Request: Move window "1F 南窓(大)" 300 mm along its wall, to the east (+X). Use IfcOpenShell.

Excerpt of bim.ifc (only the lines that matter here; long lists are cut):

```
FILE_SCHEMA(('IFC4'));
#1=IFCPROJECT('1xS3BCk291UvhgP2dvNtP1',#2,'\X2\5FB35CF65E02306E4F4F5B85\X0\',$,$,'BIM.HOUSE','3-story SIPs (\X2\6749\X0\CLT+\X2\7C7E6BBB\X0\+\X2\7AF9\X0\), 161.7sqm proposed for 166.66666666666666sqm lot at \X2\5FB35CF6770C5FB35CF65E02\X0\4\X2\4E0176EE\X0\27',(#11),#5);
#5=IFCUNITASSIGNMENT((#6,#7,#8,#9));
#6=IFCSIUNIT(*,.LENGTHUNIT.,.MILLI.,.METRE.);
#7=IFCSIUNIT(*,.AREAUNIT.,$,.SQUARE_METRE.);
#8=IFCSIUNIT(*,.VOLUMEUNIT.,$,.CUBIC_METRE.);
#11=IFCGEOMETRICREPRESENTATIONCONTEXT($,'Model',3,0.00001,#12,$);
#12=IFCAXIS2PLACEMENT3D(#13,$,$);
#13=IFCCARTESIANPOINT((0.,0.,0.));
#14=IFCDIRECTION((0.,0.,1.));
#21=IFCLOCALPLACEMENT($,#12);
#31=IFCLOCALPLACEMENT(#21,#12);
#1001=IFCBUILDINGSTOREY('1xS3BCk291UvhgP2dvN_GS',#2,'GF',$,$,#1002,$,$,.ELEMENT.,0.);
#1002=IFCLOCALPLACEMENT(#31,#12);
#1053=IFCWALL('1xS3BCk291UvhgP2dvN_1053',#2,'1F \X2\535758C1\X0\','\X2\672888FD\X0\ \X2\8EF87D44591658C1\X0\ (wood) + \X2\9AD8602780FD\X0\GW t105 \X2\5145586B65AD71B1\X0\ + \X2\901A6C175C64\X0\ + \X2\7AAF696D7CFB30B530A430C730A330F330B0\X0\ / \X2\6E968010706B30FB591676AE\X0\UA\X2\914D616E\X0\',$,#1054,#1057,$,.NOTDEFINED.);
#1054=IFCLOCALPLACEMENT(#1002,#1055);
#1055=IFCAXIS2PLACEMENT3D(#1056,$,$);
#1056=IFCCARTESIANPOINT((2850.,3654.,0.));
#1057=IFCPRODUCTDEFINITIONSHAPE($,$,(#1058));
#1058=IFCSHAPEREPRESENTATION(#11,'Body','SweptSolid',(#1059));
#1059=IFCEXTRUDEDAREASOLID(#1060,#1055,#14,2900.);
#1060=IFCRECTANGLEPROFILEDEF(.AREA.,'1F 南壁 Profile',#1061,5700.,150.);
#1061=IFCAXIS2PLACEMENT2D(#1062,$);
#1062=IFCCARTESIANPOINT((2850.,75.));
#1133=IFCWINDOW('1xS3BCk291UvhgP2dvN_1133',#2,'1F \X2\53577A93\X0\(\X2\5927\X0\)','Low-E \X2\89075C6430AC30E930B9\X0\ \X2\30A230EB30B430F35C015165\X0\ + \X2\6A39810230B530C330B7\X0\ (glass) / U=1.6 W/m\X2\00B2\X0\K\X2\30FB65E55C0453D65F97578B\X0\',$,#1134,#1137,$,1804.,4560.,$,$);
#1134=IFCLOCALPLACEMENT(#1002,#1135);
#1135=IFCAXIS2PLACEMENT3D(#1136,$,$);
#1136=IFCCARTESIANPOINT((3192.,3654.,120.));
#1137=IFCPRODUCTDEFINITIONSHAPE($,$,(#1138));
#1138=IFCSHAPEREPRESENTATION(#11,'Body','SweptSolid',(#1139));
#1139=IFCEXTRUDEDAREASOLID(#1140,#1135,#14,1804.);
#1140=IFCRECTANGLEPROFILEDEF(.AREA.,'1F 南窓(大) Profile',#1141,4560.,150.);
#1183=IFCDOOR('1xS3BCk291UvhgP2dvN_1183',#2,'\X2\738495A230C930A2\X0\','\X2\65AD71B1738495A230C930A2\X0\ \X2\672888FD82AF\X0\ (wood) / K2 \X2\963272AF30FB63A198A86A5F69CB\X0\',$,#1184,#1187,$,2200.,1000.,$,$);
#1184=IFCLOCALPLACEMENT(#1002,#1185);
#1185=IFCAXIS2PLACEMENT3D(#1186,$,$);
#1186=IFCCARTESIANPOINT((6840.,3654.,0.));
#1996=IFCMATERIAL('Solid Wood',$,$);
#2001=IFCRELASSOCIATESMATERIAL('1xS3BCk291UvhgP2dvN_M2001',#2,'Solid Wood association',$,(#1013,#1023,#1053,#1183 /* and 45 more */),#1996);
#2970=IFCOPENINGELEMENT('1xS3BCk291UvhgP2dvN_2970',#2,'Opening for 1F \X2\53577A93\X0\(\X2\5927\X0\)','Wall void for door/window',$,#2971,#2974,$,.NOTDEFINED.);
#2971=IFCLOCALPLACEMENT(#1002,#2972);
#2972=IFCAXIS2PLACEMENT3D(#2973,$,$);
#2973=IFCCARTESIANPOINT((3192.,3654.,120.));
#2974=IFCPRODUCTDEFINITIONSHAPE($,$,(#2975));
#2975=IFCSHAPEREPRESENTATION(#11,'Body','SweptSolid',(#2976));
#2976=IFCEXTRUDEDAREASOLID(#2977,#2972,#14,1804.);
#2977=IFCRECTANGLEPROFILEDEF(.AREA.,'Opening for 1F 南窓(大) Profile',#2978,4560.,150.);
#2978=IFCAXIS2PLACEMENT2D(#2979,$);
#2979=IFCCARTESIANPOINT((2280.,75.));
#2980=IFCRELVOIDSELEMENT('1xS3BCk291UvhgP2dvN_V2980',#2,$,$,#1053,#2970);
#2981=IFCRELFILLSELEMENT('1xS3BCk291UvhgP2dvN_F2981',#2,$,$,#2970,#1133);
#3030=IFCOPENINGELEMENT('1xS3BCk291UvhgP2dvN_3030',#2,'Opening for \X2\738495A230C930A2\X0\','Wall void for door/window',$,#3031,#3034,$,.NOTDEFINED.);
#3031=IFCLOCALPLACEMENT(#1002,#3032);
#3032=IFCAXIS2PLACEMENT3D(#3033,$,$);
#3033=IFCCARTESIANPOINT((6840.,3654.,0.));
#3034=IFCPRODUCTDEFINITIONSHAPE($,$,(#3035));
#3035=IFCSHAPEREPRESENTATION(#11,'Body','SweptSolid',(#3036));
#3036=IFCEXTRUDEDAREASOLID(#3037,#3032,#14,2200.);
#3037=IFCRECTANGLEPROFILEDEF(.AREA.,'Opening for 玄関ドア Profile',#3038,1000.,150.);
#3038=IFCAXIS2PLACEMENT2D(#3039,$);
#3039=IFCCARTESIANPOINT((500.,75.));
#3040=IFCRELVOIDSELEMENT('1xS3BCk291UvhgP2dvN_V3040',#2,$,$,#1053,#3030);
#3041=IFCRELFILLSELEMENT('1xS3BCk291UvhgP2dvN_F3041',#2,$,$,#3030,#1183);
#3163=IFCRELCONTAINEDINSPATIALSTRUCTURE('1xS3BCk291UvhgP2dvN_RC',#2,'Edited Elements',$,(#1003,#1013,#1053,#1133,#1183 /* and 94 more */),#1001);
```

```python
import ifcopenshell
import ifcopenshell.api.geometry
import ifcopenshell.util.placement
import ifcopenshell.util.unit

model = ifcopenshell.open("bim.ifc")
unit_scale = ifcopenshell.util.unit.calculate_unit_scale(model)

window = model.by_guid("1xS3BCk291UvhgP2dvN_1133")
opening = window.FillsVoids[0].RelatingOpeningElement
wall = opening.VoidsElements[0].RelatingBuildingElement

wall_matrix = ifcopenshell.util.placement.get_local_placement(wall.ObjectPlacement)
shift = wall_matrix[:3, 0] * 0.3 / unit_scale
before = ifcopenshell.util.placement.get_local_placement(window.ObjectPlacement)[:3, 3].copy()

# The window is not placed relative to its opening, so move both.
for product in (opening, window):
    matrix = ifcopenshell.util.placement.get_local_placement(product.ObjectPlacement)
    matrix[:3, 3] += shift
    ifcopenshell.api.geometry.edit_object_placement(model, product=product, matrix=matrix, is_si=False)

after = ifcopenshell.util.placement.get_local_placement(window.ObjectPlacement)[:3, 3]
print("window moved by", (after - before).round(3) + 0.0)

model.write("bim_edited.ifc")
```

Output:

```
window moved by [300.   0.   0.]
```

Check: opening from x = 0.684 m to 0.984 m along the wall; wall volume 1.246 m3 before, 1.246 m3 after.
